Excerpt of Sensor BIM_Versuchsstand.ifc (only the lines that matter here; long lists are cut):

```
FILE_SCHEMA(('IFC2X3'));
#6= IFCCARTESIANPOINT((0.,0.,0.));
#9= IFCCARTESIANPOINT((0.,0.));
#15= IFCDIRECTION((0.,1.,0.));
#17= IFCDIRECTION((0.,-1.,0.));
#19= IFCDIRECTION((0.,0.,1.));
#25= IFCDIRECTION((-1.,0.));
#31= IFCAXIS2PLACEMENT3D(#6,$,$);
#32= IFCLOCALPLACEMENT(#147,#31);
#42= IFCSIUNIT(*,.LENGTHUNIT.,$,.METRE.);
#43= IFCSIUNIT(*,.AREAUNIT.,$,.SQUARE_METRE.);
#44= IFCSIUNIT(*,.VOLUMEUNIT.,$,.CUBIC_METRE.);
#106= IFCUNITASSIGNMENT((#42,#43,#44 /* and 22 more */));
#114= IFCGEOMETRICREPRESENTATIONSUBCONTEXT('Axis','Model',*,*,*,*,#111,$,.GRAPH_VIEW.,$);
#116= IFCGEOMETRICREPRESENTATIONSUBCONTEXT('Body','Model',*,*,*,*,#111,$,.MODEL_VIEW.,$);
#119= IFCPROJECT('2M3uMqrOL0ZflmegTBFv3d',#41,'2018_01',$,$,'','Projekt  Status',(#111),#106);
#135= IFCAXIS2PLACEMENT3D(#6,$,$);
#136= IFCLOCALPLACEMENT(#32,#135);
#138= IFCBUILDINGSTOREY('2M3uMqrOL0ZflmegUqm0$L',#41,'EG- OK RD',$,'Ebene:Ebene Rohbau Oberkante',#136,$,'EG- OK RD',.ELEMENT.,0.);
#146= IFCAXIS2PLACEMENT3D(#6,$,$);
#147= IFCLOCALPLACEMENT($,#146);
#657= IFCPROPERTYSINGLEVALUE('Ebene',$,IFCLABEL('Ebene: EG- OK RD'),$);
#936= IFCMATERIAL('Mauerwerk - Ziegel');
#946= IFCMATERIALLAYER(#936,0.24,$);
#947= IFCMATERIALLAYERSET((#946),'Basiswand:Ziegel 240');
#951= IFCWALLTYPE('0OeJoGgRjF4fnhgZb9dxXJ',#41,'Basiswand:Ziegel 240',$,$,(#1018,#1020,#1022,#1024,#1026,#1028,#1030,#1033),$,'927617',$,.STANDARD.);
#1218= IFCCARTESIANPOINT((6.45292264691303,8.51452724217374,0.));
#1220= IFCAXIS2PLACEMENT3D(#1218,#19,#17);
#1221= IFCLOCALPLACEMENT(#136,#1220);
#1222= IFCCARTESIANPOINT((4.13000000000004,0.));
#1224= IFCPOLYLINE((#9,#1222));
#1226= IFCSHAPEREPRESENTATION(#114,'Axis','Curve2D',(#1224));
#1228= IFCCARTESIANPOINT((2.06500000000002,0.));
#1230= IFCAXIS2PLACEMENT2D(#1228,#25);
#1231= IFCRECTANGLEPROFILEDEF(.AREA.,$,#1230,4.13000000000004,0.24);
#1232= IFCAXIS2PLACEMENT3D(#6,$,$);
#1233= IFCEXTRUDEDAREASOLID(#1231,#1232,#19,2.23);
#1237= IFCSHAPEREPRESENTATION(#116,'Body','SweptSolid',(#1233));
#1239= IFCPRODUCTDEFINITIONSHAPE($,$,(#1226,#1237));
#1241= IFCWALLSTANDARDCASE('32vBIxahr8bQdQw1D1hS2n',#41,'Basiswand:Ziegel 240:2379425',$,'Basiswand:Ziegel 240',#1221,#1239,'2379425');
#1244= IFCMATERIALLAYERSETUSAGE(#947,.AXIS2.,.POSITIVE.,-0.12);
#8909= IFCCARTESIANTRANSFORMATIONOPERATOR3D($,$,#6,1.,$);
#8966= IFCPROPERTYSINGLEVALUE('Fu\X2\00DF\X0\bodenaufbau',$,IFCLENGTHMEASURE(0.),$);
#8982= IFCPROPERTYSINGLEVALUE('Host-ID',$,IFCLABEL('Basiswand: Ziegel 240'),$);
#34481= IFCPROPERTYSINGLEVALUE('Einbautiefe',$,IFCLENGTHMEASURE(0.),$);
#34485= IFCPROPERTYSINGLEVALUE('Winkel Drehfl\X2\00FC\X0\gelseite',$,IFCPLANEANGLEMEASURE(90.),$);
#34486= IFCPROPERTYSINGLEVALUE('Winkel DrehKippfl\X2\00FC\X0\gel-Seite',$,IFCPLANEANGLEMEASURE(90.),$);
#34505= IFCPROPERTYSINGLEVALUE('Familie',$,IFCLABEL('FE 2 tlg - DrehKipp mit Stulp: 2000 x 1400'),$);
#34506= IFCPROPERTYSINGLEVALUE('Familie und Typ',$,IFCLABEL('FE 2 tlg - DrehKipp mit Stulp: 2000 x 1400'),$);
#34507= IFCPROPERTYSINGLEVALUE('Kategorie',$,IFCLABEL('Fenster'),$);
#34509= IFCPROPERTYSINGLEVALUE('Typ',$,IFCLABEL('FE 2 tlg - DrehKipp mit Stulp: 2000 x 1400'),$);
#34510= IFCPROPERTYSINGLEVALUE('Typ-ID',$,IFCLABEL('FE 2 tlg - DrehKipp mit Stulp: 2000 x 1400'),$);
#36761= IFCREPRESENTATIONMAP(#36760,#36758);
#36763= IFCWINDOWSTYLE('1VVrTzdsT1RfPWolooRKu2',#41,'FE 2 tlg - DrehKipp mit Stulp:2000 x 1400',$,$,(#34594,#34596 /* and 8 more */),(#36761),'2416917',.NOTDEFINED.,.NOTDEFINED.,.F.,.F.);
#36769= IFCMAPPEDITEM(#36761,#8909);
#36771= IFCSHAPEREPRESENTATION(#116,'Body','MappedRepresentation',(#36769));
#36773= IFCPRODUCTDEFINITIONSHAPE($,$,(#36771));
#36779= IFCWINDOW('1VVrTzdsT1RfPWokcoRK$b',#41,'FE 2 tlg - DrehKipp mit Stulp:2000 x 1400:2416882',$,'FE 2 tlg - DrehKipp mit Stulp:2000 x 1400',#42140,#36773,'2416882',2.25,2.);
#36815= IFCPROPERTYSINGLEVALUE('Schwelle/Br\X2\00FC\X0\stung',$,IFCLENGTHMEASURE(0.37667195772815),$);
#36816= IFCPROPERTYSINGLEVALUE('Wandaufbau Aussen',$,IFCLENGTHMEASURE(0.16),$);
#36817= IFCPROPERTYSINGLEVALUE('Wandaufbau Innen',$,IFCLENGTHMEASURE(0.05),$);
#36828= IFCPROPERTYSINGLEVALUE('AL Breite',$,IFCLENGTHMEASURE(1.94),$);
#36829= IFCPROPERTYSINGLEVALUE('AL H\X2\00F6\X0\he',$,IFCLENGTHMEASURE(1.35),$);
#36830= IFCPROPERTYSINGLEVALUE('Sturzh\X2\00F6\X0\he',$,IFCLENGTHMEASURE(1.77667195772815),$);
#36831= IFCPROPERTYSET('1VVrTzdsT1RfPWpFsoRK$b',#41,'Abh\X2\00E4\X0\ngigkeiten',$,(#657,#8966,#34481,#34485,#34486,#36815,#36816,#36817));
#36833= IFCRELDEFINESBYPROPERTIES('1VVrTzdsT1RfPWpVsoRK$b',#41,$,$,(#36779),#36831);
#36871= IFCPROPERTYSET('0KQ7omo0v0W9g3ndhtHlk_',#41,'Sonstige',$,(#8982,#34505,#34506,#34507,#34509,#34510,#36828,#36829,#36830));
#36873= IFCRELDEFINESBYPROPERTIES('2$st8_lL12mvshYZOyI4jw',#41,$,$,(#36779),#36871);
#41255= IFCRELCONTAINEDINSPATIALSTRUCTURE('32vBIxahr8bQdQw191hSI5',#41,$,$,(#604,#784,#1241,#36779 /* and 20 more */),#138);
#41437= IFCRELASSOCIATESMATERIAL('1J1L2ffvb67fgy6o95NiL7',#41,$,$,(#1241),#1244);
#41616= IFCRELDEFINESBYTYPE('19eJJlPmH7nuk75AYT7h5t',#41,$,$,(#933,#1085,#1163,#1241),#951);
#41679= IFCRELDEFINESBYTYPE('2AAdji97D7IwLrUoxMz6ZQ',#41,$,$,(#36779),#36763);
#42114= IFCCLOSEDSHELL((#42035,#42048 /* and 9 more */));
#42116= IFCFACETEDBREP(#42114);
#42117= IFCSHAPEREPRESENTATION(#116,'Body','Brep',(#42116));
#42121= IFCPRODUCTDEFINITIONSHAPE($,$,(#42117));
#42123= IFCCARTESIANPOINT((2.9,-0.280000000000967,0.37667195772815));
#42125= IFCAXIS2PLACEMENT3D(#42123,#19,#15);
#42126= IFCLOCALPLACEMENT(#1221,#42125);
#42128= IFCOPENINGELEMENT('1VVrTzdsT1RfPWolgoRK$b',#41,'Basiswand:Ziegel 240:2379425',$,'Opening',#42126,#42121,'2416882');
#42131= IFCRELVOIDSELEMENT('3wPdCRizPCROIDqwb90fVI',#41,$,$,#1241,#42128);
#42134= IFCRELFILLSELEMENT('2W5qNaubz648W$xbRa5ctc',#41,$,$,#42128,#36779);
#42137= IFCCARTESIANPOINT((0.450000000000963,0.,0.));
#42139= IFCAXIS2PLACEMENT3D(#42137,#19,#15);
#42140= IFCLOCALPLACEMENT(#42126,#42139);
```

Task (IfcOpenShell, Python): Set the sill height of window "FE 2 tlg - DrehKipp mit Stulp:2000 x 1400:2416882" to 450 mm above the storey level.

```python
import numpy as np
import ifcopenshell
import ifcopenshell.api.geometry
import ifcopenshell.api.pset
import ifcopenshell.geom
import ifcopenshell.util.element
import ifcopenshell.util.placement
import ifcopenshell.util.shape
import ifcopenshell.util.unit

model = ifcopenshell.open("Sensor BIM_Versuchsstand.ifc")
unit_scale = ifcopenshell.util.unit.calculate_unit_scale(model)

window = model.by_guid("1VVrTzdsT1RfPWokcoRK$b")
opening = window.FillsVoids[0].RelatingOpeningElement
storey = ifcopenshell.util.element.get_container(window, ifc_class="IfcBuildingStorey")
level = ifcopenshell.util.placement.get_local_placement(storey.ObjectPlacement)[2, 3]

# The opening's origin need not be at the sill, so measure its lowest point.
shape = ifcopenshell.geom.create_shape(ifcopenshell.geom.settings(), opening)
bottom = ifcopenshell.util.shape.get_shape_bottom_elevation(shape, shape.geometry) / unit_scale
dz = level + 0.45 - bottom

shift = np.array([0.0, 0.0, dz])
# The window is placed relative to its opening, so it follows when the opening moves.
matrix = ifcopenshell.util.placement.get_local_placement(opening.ObjectPlacement)
matrix[:3, 3] += shift
ifcopenshell.api.geometry.edit_object_placement(
    model, product=opening, matrix=matrix, is_si=False, should_transform_children=True
)

# Keep the stored heights in step.
pset = model.by_id(ifcopenshell.util.element.get_pset(window, "Abhängigkeiten", should_inherit=False)["id"])
ifcopenshell.api.pset.edit_pset(model, pset=pset, properties={
    "Schwelle/Brüstung": model.create_entity("IfcLengthMeasure", ifcopenshell.util.element.get_pset(window, "Abhängigkeiten", "Schwelle/Brüstung") + dz),
})
pset = model.by_id(ifcopenshell.util.element.get_pset(window, "Sonstige", should_inherit=False)["id"])
ifcopenshell.api.pset.edit_pset(model, pset=pset, properties={
    "Sturzhöhe": model.create_entity("IfcLengthMeasure", ifcopenshell.util.element.get_pset(window, "Sonstige", "Sturzhöhe") + dz),
})

print(f"moved by {dz * unit_scale:+.3f} m")

model.write("Sensor BIM_Versuchsstand-out.ifc")
```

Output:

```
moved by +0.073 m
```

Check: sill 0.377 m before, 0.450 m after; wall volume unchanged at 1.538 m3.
